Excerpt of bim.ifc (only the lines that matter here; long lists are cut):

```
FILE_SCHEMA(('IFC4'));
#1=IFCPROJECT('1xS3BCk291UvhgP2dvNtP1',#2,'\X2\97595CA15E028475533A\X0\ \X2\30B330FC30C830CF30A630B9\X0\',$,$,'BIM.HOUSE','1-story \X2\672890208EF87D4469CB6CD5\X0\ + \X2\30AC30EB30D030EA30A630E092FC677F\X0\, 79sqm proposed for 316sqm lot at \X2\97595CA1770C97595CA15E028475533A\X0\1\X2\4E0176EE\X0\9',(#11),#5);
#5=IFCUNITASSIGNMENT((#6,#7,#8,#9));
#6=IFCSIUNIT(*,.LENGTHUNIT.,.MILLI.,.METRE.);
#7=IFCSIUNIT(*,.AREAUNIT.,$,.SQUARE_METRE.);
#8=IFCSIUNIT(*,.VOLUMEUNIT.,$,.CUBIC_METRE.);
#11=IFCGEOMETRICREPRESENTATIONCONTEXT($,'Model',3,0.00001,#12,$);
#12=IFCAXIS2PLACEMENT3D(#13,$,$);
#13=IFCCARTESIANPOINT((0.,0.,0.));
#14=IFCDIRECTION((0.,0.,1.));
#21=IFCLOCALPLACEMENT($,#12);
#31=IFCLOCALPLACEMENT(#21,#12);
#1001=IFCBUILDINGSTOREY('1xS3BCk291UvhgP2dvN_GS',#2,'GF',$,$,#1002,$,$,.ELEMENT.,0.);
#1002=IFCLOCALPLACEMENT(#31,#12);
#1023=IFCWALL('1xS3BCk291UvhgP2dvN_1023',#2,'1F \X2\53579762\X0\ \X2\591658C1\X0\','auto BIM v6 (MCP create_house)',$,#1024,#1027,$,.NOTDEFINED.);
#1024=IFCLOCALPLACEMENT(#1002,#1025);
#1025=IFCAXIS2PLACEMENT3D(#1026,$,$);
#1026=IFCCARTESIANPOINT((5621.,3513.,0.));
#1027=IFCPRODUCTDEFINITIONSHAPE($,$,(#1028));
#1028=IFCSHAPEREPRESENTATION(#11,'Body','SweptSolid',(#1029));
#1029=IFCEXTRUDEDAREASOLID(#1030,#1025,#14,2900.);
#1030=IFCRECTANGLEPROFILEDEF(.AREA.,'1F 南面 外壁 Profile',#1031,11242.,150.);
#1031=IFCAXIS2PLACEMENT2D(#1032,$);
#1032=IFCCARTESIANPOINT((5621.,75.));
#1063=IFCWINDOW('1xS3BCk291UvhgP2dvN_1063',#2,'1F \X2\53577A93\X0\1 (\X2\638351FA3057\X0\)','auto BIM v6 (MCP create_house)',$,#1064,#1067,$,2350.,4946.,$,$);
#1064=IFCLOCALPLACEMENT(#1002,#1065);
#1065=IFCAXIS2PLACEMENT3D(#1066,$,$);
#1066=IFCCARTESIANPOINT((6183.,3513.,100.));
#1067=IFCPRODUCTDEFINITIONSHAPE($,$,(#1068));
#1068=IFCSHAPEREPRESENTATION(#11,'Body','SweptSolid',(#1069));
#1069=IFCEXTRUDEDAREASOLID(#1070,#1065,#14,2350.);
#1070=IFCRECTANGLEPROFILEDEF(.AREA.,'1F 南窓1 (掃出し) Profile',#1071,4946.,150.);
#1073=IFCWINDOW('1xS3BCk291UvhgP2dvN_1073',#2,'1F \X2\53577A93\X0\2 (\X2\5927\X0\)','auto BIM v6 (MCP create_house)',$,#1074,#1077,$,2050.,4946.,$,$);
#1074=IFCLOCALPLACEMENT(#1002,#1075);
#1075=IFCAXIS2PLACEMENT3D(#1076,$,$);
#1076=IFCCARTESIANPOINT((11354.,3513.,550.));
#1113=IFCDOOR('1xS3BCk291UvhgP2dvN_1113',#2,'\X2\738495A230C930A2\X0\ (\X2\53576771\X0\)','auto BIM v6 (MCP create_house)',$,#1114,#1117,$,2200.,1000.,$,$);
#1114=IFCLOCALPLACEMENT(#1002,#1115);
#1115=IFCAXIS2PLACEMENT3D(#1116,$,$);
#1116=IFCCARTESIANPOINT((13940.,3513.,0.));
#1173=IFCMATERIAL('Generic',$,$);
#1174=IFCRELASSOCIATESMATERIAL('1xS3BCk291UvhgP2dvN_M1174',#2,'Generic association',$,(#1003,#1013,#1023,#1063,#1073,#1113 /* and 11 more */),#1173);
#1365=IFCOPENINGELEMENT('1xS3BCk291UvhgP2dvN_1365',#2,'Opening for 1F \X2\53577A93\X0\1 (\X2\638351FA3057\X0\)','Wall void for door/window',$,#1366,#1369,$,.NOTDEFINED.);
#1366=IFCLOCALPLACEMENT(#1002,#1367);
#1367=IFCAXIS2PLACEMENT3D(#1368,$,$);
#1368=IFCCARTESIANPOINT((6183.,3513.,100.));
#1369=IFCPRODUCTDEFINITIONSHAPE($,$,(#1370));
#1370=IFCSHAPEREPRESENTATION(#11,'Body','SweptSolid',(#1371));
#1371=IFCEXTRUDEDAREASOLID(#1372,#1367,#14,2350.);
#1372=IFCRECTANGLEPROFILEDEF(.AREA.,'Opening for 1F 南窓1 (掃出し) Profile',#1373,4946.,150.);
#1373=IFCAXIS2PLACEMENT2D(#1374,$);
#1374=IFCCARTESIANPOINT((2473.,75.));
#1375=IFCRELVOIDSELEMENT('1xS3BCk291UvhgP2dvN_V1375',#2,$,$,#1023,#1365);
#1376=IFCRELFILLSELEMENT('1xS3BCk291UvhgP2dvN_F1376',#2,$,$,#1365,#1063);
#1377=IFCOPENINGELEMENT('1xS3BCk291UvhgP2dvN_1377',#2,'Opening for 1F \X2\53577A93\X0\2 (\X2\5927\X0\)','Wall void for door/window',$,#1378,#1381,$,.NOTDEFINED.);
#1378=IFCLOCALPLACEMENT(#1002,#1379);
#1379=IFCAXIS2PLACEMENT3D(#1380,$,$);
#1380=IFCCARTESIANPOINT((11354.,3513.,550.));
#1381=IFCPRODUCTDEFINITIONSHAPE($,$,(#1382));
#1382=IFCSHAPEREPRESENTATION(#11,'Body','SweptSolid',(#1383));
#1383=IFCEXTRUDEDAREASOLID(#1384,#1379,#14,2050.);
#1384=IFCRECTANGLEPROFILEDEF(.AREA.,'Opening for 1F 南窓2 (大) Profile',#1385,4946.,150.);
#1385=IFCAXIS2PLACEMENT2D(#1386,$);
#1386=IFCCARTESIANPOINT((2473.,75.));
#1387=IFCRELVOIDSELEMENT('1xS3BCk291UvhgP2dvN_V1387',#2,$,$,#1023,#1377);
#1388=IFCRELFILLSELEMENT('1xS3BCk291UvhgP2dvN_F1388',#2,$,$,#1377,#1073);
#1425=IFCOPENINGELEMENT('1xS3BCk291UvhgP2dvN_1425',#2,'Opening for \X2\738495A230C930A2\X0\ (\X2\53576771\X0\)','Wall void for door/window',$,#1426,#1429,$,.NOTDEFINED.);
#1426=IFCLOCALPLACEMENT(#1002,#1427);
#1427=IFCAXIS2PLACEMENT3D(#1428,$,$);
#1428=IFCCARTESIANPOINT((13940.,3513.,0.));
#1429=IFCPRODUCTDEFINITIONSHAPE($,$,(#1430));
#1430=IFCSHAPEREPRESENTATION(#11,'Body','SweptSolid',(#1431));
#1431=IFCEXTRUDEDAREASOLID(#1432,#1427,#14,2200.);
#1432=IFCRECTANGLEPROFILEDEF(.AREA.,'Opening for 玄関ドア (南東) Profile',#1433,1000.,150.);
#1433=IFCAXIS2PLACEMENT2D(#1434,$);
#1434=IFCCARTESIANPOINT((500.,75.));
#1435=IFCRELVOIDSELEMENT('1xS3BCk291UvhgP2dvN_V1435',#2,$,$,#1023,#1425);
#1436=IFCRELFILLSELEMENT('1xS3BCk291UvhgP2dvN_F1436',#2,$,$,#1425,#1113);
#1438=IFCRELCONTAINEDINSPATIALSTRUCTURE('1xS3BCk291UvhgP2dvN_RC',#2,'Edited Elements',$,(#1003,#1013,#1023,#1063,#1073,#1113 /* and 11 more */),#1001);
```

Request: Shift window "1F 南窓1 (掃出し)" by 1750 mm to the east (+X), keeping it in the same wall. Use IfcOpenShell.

```python
import ifcopenshell
import ifcopenshell.api.geometry
import ifcopenshell.util.placement
import ifcopenshell.util.unit

model = ifcopenshell.open("bim.ifc")
unit_scale = ifcopenshell.util.unit.calculate_unit_scale(model)

window = model.by_id(1063)
opening = window.FillsVoids[0].RelatingOpeningElement
wall = opening.VoidsElements[0].RelatingBuildingElement

wall_matrix = ifcopenshell.util.placement.get_local_placement(wall.ObjectPlacement)
shift = wall_matrix[:3, 0] * 1.75 / unit_scale
before = ifcopenshell.util.placement.get_local_placement(window.ObjectPlacement)[:3, 3].copy()

# The window is not placed relative to its opening, so move both.
for product in (opening, window):
    matrix = ifcopenshell.util.placement.get_local_placement(product.ObjectPlacement)
    matrix[:3, 3] += shift
    ifcopenshell.api.geometry.edit_object_placement(model, product=product, matrix=matrix, is_si=False)

after = ifcopenshell.util.placement.get_local_placement(window.ObjectPlacement)[:3, 3]
print("window moved by", (after - before).round(3) + 0.0)

model.write("bim_rev.ifc")
```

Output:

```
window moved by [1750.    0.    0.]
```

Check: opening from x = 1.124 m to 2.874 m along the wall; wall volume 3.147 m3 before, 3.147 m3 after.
